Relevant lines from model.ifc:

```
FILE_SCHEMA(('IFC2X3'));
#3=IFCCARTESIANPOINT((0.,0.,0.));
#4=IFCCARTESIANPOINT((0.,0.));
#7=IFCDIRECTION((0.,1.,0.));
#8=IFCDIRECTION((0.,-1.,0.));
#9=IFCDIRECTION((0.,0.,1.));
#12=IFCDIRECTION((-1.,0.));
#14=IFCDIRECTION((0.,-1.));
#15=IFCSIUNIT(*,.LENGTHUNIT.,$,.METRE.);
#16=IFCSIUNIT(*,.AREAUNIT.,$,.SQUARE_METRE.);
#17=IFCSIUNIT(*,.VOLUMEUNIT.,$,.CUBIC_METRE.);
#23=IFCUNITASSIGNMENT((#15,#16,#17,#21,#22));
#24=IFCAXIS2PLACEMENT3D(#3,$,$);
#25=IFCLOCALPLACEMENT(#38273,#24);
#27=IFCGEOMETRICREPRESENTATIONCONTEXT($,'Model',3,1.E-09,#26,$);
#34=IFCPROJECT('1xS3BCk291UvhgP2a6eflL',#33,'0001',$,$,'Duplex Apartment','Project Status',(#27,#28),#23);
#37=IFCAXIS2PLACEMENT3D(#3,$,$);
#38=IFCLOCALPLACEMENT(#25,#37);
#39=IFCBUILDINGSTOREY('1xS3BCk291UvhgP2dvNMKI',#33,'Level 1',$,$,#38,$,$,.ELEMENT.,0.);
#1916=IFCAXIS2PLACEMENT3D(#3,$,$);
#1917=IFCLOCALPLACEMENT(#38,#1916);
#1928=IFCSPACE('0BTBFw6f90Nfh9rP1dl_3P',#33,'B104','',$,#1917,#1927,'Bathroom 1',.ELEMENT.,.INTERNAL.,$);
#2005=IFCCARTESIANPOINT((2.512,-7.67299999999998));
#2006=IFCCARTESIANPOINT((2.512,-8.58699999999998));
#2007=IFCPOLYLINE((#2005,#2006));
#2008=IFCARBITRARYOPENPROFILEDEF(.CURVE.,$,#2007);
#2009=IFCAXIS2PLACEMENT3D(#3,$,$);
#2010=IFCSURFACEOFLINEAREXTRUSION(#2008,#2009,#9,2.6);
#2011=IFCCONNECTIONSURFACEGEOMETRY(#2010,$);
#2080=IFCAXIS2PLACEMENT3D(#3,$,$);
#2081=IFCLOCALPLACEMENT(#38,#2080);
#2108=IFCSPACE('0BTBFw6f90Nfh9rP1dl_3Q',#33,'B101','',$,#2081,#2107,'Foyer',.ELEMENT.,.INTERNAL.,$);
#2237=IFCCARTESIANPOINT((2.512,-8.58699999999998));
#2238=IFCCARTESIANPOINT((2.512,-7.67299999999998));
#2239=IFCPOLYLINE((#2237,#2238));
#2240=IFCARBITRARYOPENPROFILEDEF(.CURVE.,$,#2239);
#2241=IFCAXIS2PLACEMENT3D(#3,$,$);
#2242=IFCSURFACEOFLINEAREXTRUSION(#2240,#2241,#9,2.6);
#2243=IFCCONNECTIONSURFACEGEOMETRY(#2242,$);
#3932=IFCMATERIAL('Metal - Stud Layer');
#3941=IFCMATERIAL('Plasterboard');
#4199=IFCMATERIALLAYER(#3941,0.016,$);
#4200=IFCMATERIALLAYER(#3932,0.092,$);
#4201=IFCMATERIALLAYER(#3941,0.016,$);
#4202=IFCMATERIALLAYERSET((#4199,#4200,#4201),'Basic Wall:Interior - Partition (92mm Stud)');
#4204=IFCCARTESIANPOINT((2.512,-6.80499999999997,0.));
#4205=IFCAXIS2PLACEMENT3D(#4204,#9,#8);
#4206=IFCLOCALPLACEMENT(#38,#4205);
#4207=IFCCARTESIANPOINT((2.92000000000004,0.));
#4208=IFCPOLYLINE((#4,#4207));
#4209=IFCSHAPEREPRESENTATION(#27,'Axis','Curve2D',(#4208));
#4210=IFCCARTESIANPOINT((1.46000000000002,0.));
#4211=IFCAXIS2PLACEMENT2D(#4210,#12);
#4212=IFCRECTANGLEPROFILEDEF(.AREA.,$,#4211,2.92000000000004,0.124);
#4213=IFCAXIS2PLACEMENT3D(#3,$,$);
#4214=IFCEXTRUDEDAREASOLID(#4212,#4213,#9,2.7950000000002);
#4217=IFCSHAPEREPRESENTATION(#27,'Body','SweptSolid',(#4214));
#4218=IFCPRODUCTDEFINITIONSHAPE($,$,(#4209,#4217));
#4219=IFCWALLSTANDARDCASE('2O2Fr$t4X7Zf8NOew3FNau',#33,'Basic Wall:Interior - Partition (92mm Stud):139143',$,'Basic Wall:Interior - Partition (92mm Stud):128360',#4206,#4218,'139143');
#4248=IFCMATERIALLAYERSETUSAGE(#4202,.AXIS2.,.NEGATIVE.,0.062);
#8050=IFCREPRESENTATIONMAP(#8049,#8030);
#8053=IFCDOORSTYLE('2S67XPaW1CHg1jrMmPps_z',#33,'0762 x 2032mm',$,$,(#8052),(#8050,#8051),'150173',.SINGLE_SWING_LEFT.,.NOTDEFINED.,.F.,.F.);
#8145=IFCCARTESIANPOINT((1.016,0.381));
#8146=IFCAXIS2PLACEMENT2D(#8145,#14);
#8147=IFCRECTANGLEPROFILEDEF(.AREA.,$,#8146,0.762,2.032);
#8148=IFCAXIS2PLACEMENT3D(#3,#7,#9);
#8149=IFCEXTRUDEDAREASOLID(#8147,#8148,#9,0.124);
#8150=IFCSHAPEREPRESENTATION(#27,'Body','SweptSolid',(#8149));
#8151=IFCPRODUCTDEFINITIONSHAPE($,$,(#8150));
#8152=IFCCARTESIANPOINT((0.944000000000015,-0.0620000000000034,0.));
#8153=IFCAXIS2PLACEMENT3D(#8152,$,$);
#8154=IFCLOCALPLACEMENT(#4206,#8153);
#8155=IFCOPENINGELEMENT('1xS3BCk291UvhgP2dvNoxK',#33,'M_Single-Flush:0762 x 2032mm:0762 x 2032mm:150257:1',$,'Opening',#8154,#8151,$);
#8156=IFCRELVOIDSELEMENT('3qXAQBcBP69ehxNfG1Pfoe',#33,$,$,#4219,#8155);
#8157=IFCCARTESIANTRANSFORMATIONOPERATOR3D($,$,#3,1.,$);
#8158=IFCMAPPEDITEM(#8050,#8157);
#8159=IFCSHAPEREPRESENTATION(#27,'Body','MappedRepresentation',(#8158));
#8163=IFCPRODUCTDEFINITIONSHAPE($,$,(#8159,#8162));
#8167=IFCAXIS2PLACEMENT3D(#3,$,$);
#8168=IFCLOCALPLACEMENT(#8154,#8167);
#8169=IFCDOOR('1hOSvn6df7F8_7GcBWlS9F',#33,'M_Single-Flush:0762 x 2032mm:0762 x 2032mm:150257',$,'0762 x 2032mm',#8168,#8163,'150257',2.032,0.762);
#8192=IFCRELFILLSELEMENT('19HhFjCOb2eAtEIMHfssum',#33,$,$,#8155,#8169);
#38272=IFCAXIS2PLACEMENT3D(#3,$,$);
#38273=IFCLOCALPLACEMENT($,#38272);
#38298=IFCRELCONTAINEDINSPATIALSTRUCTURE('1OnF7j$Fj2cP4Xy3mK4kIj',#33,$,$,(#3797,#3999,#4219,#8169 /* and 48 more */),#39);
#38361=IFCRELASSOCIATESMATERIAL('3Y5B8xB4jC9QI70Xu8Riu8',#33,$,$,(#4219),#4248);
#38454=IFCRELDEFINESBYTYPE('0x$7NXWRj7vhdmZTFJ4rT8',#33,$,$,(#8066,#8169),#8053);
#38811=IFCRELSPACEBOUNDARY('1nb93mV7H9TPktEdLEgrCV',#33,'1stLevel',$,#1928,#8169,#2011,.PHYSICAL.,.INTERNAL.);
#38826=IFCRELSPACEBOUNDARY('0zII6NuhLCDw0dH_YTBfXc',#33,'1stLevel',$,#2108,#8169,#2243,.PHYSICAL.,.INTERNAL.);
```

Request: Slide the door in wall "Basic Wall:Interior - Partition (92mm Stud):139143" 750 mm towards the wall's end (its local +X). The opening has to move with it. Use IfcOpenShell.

```python
import numpy as np
import ifcopenshell
import ifcopenshell.api.geometry
import ifcopenshell.util.placement

model = ifcopenshell.open("model.ifc")

door = model.by_id(8169)
opening = door.FillsVoids[0].RelatingOpeningElement
wall = opening.VoidsElements[0].RelatingBuildingElement

wall_matrix = ifcopenshell.util.placement.get_local_placement(wall.ObjectPlacement)
shift = wall_matrix[:3, 0] * 0.75
before = ifcopenshell.util.placement.get_local_placement(door.ObjectPlacement)[:3, 3].copy()

# The door is placed relative to its opening, so it follows when the opening moves.
matrix = ifcopenshell.util.placement.get_local_placement(opening.ObjectPlacement)
matrix[:3, 3] += shift
ifcopenshell.api.geometry.edit_object_placement(
    model, product=opening, matrix=matrix, is_si=False, should_transform_children=True
)

# Space boundary surfaces are stored in each space's coordinates; move them too.
for rel in door.ProvidesBoundaries:
    if not rel.ConnectionGeometry:
        continue
    surface = rel.ConnectionGeometry.SurfaceOnRelatingElement
    space_matrix = ifcopenshell.util.placement.get_local_placement(rel.RelatingSpace.ObjectPlacement)
    point = np.array(surface.Position.Location.Coordinates) + space_matrix[:3, :3].T @ shift
    surface.Position = model.createIfcAxis2Placement3D(
        model.createIfcCartesianPoint(point.tolist()), surface.Position.Axis, surface.Position.RefDirection
    )

after = ifcopenshell.util.placement.get_local_placement(door.ObjectPlacement)[:3, 3]
print("door moved by", (after - before).round(3) + 0.0)

model.write("model_edited.ifc")
```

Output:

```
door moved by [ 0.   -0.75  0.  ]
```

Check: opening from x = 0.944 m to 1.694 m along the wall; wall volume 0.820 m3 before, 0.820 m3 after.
